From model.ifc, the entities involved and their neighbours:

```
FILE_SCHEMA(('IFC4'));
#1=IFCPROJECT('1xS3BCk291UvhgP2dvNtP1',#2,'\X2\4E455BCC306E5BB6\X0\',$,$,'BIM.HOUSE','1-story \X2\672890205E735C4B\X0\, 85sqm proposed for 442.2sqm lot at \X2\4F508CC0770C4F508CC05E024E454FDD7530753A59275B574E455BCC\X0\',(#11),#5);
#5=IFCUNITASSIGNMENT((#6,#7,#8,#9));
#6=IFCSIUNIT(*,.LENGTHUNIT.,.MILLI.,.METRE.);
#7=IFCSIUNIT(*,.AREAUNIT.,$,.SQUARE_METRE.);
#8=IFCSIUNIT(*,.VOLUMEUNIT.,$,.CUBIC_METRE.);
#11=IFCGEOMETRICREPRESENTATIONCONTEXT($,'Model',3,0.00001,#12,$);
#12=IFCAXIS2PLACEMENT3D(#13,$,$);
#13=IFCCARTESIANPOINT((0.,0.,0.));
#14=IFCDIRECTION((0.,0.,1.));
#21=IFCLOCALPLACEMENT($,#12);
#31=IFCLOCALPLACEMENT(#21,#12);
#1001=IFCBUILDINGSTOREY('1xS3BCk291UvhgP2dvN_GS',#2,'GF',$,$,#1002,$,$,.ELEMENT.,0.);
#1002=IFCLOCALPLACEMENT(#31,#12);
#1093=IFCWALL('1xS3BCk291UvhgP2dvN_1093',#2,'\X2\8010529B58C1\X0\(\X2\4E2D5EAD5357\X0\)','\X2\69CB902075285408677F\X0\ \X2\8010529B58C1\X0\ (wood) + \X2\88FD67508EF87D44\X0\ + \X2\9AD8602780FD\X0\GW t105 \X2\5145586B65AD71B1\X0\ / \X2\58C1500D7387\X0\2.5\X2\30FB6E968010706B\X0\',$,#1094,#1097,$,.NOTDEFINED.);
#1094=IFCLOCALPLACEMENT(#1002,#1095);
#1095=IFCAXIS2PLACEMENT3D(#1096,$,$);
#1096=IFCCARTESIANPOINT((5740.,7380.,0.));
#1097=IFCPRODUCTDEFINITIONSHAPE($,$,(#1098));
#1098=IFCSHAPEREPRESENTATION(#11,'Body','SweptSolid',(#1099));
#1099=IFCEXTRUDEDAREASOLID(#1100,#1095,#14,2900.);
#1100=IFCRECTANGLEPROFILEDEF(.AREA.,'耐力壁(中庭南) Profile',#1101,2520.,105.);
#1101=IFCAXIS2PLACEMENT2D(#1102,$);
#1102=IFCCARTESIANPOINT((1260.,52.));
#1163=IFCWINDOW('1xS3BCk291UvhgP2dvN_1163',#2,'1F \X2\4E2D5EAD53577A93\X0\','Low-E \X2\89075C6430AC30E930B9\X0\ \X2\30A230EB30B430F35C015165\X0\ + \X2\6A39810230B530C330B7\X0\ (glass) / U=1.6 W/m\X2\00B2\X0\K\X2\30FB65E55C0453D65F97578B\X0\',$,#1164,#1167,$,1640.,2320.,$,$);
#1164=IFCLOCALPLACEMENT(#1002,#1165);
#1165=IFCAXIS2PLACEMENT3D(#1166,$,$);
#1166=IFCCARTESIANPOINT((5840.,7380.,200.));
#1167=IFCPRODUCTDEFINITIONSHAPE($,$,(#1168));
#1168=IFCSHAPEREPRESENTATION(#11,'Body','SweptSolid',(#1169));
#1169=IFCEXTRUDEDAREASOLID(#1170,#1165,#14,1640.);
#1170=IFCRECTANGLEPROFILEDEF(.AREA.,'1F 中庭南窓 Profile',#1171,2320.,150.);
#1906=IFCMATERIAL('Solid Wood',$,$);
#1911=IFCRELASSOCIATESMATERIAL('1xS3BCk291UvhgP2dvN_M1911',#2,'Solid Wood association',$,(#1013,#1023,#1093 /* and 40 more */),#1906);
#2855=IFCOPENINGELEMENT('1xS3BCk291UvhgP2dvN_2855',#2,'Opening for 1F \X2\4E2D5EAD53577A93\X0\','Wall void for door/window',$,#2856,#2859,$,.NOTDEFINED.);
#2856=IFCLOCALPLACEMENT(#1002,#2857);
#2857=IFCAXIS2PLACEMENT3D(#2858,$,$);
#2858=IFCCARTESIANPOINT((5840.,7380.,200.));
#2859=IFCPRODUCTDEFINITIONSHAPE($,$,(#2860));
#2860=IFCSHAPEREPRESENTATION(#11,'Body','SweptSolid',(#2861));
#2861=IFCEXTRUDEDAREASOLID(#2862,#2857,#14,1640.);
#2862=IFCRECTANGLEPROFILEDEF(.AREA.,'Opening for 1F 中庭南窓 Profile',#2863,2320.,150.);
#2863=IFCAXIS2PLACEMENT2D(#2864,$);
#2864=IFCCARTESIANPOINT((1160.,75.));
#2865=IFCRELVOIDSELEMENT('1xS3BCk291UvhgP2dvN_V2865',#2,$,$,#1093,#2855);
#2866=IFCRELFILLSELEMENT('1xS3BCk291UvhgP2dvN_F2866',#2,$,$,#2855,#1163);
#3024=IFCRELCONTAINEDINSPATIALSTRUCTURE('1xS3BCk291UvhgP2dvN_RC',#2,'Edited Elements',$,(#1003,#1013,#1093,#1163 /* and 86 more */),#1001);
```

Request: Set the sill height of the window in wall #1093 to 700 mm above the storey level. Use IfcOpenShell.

```python
import numpy as np
import ifcopenshell
import ifcopenshell.api.geometry
import ifcopenshell.geom
import ifcopenshell.util.element
import ifcopenshell.util.placement
import ifcopenshell.util.shape
import ifcopenshell.util.unit

model = ifcopenshell.open("model.ifc")
unit_scale = ifcopenshell.util.unit.calculate_unit_scale(model)

window = model.by_guid("1xS3BCk291UvhgP2dvN_1163")
opening = window.FillsVoids[0].RelatingOpeningElement
storey = ifcopenshell.util.element.get_container(window, ifc_class="IfcBuildingStorey")
level = ifcopenshell.util.placement.get_local_placement(storey.ObjectPlacement)[2, 3]

# The opening's origin need not be at the sill, so measure its lowest point.
shape = ifcopenshell.geom.create_shape(ifcopenshell.geom.settings(), opening)
bottom = ifcopenshell.util.shape.get_shape_bottom_elevation(shape, shape.geometry) / unit_scale
dz = level + 0.7 / unit_scale - bottom

shift = np.array([0.0, 0.0, dz])
# The window is not placed relative to its opening, so move both.
for product in (opening, window):
    matrix = ifcopenshell.util.placement.get_local_placement(product.ObjectPlacement)
    matrix[:3, 3] += shift
    ifcopenshell.api.geometry.edit_object_placement(model, product=product, matrix=matrix, is_si=False)

print(f"moved by {dz * unit_scale:+.3f} m")

model.write("model-out.ifc")
```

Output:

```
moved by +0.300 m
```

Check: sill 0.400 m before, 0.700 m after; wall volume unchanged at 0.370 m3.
